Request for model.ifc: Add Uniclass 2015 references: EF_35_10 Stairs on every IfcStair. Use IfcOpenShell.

First a look at what the model holds.

```python
import ifcopenshell

model = ifcopenshell.open("model.ifc")
print(model.schema)
print("classifications:", [c.Name for c in model.by_type("IfcClassification")])
for ifc_class in ("IfcDoor", "IfcRoof", "IfcStair", "IfcWall", "IfcWindow"):
    print(ifc_class, len(model.by_type(ifc_class)))
```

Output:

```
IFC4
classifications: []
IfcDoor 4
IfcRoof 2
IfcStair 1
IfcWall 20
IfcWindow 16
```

```python
import ifcopenshell
import ifcopenshell.api.classification

model = ifcopenshell.open("model.ifc")

system = ifcopenshell.api.classification.add_classification(model, classification="Uniclass 2015")

codes = {
    "IfcStair": ("EF_35_10", "Stairs"),
}
for ifc_class, (code, name) in codes.items():
    products = model.by_type(ifc_class)
    ifcopenshell.api.classification.add_reference(
        model, products=products, classification=system, identification=code, name=name
    )
    print(code, len(products))

model.write("model_v2.ifc")
```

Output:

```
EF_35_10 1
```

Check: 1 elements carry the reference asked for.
